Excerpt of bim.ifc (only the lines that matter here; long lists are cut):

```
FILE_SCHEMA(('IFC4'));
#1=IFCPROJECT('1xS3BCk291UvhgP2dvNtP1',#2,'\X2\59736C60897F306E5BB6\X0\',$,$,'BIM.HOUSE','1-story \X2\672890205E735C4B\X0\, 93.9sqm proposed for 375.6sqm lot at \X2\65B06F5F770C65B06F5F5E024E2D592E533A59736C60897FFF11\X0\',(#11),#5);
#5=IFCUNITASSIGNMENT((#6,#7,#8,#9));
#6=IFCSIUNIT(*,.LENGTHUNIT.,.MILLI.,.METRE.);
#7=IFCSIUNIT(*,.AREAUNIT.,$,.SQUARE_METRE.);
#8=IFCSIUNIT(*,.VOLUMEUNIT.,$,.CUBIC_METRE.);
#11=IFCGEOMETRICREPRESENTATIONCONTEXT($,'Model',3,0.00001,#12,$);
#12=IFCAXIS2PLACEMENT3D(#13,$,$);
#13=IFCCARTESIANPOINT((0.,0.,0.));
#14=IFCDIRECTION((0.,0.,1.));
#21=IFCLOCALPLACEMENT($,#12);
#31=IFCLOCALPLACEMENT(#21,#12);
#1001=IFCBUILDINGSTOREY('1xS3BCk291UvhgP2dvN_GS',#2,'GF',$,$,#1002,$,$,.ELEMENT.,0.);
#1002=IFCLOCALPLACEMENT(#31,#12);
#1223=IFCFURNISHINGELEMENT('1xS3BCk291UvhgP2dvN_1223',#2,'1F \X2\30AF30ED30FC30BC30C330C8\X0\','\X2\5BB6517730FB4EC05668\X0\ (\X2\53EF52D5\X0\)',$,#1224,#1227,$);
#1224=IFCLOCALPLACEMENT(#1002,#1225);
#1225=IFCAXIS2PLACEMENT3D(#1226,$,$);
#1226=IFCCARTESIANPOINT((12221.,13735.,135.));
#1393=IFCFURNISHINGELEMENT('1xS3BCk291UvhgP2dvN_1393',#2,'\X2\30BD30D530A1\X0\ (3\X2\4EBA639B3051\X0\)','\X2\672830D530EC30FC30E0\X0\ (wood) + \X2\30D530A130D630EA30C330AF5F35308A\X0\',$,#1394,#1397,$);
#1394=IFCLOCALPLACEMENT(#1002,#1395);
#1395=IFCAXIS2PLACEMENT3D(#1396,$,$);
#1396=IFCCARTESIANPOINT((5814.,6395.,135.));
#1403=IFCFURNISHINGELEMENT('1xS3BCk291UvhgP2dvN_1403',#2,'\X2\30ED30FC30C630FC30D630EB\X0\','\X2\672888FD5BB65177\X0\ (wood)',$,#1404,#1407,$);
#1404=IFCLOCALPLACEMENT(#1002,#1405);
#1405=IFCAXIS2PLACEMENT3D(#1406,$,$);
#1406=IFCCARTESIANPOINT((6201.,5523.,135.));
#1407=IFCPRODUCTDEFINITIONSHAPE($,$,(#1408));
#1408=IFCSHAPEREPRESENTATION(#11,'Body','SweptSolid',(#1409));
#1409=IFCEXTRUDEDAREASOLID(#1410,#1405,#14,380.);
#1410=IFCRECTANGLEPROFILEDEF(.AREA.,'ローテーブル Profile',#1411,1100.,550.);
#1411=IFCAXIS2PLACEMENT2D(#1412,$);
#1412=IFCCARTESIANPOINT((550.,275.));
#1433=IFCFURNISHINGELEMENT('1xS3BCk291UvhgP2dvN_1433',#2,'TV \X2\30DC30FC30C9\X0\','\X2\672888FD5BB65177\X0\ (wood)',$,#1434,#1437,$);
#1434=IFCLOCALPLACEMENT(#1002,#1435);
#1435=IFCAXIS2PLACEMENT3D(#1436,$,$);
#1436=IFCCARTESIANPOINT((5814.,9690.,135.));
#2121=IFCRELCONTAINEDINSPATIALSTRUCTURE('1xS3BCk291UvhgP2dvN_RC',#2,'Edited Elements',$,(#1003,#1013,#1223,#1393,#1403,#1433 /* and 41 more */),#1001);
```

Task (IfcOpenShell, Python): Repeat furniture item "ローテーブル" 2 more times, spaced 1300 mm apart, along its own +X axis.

```python
import ifcopenshell
import ifcopenshell.api.geometry
import ifcopenshell.api.root
import ifcopenshell.util.element
import ifcopenshell.util.placement
import ifcopenshell.util.unit

model = ifcopenshell.open("bim.ifc")
unit_scale = ifcopenshell.util.unit.calculate_unit_scale(model)


def reuse_history(source, copy):
    """copy_class also copies each property set's owner history, people and application; keep the originals."""
    for rel in copy.IsDefinedBy:
        if rel.is_a("IfcRelDefinesByProperties") and (history := rel.RelatingPropertyDefinition.OwnerHistory):
            rel.RelatingPropertyDefinition.OwnerHistory = source.OwnerHistory
            ifcopenshell.util.element.remove_deep2(model, history)


source = model.by_guid("1xS3BCk291UvhgP2dvN_1403")
base = ifcopenshell.util.placement.get_local_placement(source.ObjectPlacement)
step = base[:3, 0] * 1.3 / unit_scale

for i in range(1, 3):
    copy = ifcopenshell.api.root.copy_class(model, product=source)
    copy.Representation = ifcopenshell.util.element.copy_deep(
        model, source.Representation, exclude=["IfcGeometricRepresentationContext", "IfcRepresentationMap"]
    )
    reuse_history(source, copy)
    matrix = base.copy()
    matrix[:3, 3] += i * step
    print("added at", matrix[:3, 3].round(3) + 0.0)
    ifcopenshell.api.geometry.edit_object_placement(model, product=copy, matrix=matrix, is_si=False)

model.write("bim-out.ifc")
```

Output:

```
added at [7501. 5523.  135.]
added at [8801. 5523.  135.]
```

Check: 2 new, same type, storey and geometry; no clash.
